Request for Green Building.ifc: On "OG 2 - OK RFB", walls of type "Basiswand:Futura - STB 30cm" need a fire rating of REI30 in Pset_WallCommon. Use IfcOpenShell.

First a look at what the model holds.

```python
import ifcopenshell
import ifcopenshell.util.element

model = ifcopenshell.open("Green Building.ifc")
print(model.schema)
storey = next(s for s in model.by_type("IfcBuildingStorey") if s.Name == "OG 2 - OK RFB")
walls = [e for e in ifcopenshell.util.element.get_decomposition(storey) if e.is_a("IfcWall")]
seen = {}
for e in walls:
    element_type = ifcopenshell.util.element.get_type(e)
    key = (element_type.Name if element_type != e and element_type else None, ifcopenshell.util.element.get_pset(e, "Pset_WallCommon", "FireRating"))
    seen[key] = seen.get(key, 0) + 1
for (name, value), count in sorted(seen.items(), key=str):
    print(count, "x", name, "|", value)
```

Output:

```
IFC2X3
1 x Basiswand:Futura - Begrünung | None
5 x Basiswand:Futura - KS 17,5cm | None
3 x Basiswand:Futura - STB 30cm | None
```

```python
import ifcopenshell
import ifcopenshell.api.pset
import ifcopenshell.util.element

model = ifcopenshell.open("Green Building.ifc")

storey = next(s for s in model.by_type("IfcBuildingStorey") if s.Name == "OG 2 - OK RFB")
walls = [e for e in ifcopenshell.util.element.get_decomposition(storey) if e.is_a("IfcWall")]

count = 0
for e in walls:
    element_type = ifcopenshell.util.element.get_type(e)
    if element_type in (None, e) or element_type.Name != "Basiswand:Futura - STB 30cm":
        continue
    # add_pset returns the element's existing set when there is one.
    pset = ifcopenshell.api.pset.add_pset(model, product=e, name="Pset_WallCommon")
    ifcopenshell.api.pset.edit_pset(model, pset=pset, properties={"FireRating": "REI30"})
    count += 1

print(count, "walls updated")

model.write("Green Building-out.ifc")
```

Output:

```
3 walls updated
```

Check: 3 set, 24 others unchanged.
